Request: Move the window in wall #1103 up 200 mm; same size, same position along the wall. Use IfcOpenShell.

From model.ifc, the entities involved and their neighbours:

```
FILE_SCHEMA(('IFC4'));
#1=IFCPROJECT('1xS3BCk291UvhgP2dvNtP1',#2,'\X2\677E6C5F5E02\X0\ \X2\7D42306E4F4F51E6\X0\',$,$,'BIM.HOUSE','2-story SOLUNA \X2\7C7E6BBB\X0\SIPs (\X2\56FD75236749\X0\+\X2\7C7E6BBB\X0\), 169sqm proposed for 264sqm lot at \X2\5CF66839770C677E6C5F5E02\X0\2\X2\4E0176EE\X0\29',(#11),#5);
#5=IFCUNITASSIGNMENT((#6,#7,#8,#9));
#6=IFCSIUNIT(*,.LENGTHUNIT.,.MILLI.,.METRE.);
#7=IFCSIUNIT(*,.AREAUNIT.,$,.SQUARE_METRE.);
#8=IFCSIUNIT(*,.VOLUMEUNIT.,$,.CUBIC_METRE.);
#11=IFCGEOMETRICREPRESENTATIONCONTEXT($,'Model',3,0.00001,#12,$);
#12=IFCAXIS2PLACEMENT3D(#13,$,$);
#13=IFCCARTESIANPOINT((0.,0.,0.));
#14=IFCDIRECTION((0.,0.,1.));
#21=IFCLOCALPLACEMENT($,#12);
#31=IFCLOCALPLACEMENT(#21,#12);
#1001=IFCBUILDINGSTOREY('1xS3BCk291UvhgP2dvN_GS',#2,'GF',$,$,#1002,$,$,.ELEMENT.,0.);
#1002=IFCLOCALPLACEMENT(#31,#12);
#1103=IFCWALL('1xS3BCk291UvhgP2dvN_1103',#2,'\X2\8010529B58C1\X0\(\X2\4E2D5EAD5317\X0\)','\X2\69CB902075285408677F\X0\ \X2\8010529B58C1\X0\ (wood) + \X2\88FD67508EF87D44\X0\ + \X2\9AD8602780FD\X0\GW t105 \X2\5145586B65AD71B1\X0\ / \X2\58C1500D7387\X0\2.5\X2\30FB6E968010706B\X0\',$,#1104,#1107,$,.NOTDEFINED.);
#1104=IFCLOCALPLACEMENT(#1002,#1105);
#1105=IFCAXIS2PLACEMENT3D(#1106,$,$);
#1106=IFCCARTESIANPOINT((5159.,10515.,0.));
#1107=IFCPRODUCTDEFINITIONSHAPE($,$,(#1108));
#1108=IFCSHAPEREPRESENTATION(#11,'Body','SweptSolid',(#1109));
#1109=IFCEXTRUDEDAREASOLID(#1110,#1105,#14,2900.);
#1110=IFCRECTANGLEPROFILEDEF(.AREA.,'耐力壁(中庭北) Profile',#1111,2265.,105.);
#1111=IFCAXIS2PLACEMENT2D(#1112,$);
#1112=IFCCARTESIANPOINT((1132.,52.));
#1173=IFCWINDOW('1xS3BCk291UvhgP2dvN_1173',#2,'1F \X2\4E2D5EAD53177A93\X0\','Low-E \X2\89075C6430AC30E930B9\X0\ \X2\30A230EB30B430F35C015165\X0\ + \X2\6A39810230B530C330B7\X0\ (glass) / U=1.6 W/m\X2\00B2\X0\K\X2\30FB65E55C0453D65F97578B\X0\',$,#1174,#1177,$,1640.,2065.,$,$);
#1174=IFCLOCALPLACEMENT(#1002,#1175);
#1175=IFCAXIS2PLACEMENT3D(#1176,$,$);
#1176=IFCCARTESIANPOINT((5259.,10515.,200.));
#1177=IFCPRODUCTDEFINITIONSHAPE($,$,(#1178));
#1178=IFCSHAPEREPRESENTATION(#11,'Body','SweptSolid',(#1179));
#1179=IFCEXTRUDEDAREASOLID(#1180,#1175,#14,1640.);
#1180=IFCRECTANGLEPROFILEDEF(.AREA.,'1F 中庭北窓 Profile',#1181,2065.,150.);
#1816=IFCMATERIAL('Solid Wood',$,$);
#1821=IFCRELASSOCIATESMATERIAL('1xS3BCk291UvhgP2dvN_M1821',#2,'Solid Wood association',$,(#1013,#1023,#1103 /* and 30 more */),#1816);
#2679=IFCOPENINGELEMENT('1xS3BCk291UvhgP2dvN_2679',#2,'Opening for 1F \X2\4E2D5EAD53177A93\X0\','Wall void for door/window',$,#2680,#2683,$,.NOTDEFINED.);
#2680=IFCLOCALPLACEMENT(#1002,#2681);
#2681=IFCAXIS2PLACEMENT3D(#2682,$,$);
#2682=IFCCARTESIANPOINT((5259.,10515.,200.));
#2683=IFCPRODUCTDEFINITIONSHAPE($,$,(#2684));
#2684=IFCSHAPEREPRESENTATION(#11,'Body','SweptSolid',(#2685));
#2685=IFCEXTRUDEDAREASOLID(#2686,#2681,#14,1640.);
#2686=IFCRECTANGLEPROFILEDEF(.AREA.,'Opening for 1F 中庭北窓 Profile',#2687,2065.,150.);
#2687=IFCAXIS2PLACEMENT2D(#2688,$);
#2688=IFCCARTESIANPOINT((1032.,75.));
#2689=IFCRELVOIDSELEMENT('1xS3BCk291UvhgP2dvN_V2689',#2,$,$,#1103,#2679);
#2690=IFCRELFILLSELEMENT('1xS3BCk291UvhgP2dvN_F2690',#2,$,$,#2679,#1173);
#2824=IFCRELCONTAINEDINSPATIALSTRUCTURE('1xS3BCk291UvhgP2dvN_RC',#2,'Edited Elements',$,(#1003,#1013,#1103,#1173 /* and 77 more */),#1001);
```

```python
import numpy as np
import ifcopenshell
import ifcopenshell.api.geometry
import ifcopenshell.util.placement
import ifcopenshell.util.unit

model = ifcopenshell.open("model.ifc")
unit_scale = ifcopenshell.util.unit.calculate_unit_scale(model)

window = model.by_guid("1xS3BCk291UvhgP2dvN_1173")
opening = window.FillsVoids[0].RelatingOpeningElement
dz = 200.0

shift = np.array([0.0, 0.0, dz])
# The window is not placed relative to its opening, so move both.
for product in (opening, window):
    matrix = ifcopenshell.util.placement.get_local_placement(product.ObjectPlacement)
    matrix[:3, 3] += shift
    ifcopenshell.api.geometry.edit_object_placement(model, product=product, matrix=matrix, is_si=False)

print(f"moved by {dz * unit_scale:+.3f} m")

model.write("model-out.ifc")
```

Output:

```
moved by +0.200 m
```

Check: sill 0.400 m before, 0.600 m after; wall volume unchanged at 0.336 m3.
